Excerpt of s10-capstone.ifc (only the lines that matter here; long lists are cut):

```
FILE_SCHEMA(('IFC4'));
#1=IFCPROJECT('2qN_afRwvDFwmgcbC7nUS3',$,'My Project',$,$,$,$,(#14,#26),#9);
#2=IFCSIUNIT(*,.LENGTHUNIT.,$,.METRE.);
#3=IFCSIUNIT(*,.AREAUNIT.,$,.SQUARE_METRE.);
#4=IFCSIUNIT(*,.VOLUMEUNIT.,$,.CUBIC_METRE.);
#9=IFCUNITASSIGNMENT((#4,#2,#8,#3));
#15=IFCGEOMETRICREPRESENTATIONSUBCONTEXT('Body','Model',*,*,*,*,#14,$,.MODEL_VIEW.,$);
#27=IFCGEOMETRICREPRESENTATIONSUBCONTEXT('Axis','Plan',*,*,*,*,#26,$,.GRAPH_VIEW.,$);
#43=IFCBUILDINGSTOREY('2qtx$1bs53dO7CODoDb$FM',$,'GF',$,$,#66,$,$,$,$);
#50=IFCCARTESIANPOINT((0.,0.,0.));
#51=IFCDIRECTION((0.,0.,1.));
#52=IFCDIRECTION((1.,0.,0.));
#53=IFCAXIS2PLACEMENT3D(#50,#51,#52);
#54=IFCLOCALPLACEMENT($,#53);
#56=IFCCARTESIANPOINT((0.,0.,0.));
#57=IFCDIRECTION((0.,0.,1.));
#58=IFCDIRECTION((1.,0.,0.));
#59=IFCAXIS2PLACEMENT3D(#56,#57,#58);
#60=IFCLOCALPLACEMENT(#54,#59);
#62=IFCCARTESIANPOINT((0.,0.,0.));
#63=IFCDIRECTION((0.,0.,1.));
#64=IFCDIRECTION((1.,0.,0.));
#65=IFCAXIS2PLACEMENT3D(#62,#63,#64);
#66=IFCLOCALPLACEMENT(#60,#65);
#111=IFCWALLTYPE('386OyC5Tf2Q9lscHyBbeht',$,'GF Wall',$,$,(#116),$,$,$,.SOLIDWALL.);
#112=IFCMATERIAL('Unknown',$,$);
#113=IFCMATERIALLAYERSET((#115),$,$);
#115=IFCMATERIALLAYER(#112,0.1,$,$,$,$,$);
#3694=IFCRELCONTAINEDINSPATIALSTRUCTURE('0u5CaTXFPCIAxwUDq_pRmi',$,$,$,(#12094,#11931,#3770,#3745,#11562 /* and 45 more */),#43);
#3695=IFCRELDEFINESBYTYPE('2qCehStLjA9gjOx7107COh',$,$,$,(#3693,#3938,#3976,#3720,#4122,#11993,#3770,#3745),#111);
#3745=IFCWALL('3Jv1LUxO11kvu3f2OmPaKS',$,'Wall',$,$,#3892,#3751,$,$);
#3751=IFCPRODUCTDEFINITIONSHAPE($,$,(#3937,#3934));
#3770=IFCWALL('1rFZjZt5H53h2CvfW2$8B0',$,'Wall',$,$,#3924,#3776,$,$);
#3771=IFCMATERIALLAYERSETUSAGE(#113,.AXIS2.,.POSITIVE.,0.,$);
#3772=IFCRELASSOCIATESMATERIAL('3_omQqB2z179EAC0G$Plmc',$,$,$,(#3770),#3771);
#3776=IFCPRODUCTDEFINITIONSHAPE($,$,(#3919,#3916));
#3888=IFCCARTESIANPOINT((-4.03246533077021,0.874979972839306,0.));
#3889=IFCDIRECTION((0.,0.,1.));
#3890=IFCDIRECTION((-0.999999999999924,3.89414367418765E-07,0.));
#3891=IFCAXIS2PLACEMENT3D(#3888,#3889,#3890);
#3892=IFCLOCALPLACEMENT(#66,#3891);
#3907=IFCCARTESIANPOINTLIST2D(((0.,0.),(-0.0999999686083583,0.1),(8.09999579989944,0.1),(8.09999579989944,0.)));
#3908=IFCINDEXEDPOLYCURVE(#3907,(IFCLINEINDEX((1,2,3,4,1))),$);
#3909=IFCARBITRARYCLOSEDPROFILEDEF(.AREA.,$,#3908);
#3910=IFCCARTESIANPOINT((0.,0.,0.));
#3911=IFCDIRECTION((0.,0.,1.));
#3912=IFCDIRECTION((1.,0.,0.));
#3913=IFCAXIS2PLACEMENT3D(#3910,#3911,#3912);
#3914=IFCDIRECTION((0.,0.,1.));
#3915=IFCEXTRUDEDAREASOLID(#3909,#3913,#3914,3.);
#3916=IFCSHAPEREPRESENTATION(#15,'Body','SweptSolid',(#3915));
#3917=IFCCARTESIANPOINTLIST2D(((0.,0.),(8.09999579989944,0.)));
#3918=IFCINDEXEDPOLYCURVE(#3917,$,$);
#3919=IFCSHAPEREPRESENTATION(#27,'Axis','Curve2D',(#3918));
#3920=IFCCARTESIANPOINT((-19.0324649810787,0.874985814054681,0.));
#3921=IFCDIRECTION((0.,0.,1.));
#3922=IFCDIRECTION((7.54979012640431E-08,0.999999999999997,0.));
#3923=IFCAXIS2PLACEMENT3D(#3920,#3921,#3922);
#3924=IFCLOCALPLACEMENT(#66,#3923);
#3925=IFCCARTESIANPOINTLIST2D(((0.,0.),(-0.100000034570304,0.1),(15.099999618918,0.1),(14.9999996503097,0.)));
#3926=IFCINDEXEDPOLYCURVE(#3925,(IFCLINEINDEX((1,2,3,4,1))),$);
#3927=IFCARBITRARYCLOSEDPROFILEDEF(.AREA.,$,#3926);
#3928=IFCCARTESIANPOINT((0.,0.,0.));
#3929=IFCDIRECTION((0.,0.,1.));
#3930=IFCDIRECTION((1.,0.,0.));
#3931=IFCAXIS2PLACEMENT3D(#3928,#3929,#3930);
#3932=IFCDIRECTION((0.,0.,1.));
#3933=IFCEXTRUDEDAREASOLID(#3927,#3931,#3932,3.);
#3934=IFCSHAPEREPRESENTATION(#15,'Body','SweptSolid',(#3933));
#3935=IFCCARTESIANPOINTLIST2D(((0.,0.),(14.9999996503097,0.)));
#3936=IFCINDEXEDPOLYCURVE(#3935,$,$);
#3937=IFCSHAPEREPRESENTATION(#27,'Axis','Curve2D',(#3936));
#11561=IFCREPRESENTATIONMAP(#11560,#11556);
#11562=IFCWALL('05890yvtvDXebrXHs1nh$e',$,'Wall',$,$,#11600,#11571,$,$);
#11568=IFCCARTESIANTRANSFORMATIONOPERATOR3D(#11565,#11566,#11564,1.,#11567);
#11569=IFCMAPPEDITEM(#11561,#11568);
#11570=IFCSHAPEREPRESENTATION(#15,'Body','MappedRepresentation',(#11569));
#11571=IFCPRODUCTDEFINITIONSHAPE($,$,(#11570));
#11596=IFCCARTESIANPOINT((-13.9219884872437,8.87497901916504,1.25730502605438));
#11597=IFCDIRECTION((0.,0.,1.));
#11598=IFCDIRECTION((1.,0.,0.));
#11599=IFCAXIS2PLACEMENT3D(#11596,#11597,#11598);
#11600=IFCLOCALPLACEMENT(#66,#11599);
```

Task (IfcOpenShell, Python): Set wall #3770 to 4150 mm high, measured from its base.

```python
import ifcopenshell
import ifcopenshell.geom
import ifcopenshell.util.representation
import ifcopenshell.util.shape
import ifcopenshell.util.unit

model = ifcopenshell.open("s10-capstone.ifc")
unit_scale = ifcopenshell.util.unit.calculate_unit_scale(model)
settings = ifcopenshell.geom.settings()


def volume(element):
    """Net volume in cubic metres, openings subtracted."""
    shape = ifcopenshell.geom.create_shape(settings, element)
    return ifcopenshell.util.shape.get_volume(shape.geometry)


wall = model.by_guid("1rFZjZt5H53h2CvfW2$8B0")
before = volume(wall)

body = ifcopenshell.util.representation.get_representation(wall, "Model", "Body")
solid = body.Items[0]
old_height = solid.Depth
solid.Depth = 4.15 / unit_scale
after = volume(wall)

print(f"height {old_height:g} -> {solid.Depth:g}, volume {before:.3f} -> {after:.3f} m3")

model.write("s10-capstone_updated.ifc")
```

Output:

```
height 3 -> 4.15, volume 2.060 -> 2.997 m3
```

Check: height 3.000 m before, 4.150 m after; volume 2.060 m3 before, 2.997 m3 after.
